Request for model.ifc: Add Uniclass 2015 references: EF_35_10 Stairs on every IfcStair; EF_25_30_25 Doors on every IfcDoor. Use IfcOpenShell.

First a look at what the model holds.

```python
import ifcopenshell

model = ifcopenshell.open("model.ifc")
print(model.schema)
print("classifications:", [c.Name for c in model.by_type("IfcClassification")])
for ifc_class in ("IfcDoor", "IfcRoof", "IfcStair", "IfcWall", "IfcWindow"):
    print(ifc_class, len(model.by_type(ifc_class)))
```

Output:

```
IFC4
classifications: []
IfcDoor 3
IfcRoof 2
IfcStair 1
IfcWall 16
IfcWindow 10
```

```python
import ifcopenshell
import ifcopenshell.api.classification

model = ifcopenshell.open("model.ifc")

system = ifcopenshell.api.classification.add_classification(model, classification="Uniclass 2015")

codes = {
    "IfcStair": ("EF_35_10", "Stairs"),
    "IfcDoor": ("EF_25_30_25", "Doors"),
}
for ifc_class, (code, name) in codes.items():
    products = model.by_type(ifc_class)
    ifcopenshell.api.classification.add_reference(
        model, products=products, classification=system, identification=code, name=name
    )
    print(code, len(products))

model.write("model_v2.ifc")
```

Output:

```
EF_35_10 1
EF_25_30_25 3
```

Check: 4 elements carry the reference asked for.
